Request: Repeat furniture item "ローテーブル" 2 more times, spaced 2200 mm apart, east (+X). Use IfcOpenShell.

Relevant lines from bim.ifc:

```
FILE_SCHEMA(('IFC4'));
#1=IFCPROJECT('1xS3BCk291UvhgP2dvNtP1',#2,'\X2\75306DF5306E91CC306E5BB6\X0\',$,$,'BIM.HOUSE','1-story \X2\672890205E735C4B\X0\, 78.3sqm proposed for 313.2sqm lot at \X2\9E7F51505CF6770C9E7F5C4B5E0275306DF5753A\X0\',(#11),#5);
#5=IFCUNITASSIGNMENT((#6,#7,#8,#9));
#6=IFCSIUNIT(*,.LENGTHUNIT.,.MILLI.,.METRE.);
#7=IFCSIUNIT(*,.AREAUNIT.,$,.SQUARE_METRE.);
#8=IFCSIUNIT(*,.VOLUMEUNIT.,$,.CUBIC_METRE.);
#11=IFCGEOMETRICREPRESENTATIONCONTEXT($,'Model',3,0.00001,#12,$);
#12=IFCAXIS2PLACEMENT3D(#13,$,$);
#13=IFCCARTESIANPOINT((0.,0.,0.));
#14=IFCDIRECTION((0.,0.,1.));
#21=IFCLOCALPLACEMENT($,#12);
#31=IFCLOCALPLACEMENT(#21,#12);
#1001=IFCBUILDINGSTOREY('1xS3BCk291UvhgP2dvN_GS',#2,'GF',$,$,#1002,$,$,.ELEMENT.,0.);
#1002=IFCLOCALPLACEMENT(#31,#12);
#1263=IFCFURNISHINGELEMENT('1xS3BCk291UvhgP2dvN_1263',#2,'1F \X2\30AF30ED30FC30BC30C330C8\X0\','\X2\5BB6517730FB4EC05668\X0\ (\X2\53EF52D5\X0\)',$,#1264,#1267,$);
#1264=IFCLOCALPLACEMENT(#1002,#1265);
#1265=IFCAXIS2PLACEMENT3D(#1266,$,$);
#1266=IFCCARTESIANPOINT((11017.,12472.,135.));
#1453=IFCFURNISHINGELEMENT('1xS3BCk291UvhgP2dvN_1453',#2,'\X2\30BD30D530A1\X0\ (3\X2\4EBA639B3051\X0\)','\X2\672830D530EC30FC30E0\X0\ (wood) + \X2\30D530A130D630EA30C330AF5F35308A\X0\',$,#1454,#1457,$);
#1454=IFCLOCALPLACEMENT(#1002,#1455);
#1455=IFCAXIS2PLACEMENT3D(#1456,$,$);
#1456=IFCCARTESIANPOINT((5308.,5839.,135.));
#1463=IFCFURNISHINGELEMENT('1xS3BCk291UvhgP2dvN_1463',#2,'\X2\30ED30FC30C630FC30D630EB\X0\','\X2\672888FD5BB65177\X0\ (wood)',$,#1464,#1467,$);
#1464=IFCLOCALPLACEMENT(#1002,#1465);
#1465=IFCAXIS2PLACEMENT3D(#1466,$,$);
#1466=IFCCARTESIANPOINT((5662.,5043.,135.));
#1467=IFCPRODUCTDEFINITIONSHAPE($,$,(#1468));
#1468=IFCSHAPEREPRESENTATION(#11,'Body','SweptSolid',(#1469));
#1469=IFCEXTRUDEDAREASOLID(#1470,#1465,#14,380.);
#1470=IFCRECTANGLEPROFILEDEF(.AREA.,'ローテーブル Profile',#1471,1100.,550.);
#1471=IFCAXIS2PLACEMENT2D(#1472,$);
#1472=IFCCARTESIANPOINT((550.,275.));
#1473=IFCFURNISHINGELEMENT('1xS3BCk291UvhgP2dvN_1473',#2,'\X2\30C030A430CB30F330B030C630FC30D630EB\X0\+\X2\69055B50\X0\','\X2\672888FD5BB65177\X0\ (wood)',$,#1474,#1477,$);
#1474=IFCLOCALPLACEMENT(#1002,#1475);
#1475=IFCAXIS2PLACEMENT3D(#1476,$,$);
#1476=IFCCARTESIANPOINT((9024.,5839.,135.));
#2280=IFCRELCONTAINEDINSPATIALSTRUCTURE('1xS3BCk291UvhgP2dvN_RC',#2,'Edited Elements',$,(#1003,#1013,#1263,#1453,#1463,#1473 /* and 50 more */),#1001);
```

```python
import numpy as np
import ifcopenshell
import ifcopenshell.api.geometry
import ifcopenshell.api.root
import ifcopenshell.util.element
import ifcopenshell.util.placement

model = ifcopenshell.open("bim.ifc")


def reuse_history(source, copy):
    """copy_class also copies each property set's owner history, people and application; keep the originals."""
    for rel in copy.IsDefinedBy:
        if rel.is_a("IfcRelDefinesByProperties") and (history := rel.RelatingPropertyDefinition.OwnerHistory):
            rel.RelatingPropertyDefinition.OwnerHistory = source.OwnerHistory
            ifcopenshell.util.element.remove_deep2(model, history)


source = model.by_guid("1xS3BCk291UvhgP2dvN_1463")
base = ifcopenshell.util.placement.get_local_placement(source.ObjectPlacement)
step = np.array([1.0, 0.0, 0.0]) * 2200.0

for i in range(1, 3):
    copy = ifcopenshell.api.root.copy_class(model, product=source)
    copy.Representation = ifcopenshell.util.element.copy_deep(
        model, source.Representation, exclude=["IfcGeometricRepresentationContext", "IfcRepresentationMap"]
    )
    reuse_history(source, copy)
    matrix = base.copy()
    matrix[:3, 3] += i * step
    print("added at", matrix[:3, 3].round(3) + 0.0)
    ifcopenshell.api.geometry.edit_object_placement(model, product=copy, matrix=matrix, is_si=False)

model.write("bim-out.ifc")
```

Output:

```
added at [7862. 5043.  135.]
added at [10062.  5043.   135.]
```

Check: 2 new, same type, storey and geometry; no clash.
